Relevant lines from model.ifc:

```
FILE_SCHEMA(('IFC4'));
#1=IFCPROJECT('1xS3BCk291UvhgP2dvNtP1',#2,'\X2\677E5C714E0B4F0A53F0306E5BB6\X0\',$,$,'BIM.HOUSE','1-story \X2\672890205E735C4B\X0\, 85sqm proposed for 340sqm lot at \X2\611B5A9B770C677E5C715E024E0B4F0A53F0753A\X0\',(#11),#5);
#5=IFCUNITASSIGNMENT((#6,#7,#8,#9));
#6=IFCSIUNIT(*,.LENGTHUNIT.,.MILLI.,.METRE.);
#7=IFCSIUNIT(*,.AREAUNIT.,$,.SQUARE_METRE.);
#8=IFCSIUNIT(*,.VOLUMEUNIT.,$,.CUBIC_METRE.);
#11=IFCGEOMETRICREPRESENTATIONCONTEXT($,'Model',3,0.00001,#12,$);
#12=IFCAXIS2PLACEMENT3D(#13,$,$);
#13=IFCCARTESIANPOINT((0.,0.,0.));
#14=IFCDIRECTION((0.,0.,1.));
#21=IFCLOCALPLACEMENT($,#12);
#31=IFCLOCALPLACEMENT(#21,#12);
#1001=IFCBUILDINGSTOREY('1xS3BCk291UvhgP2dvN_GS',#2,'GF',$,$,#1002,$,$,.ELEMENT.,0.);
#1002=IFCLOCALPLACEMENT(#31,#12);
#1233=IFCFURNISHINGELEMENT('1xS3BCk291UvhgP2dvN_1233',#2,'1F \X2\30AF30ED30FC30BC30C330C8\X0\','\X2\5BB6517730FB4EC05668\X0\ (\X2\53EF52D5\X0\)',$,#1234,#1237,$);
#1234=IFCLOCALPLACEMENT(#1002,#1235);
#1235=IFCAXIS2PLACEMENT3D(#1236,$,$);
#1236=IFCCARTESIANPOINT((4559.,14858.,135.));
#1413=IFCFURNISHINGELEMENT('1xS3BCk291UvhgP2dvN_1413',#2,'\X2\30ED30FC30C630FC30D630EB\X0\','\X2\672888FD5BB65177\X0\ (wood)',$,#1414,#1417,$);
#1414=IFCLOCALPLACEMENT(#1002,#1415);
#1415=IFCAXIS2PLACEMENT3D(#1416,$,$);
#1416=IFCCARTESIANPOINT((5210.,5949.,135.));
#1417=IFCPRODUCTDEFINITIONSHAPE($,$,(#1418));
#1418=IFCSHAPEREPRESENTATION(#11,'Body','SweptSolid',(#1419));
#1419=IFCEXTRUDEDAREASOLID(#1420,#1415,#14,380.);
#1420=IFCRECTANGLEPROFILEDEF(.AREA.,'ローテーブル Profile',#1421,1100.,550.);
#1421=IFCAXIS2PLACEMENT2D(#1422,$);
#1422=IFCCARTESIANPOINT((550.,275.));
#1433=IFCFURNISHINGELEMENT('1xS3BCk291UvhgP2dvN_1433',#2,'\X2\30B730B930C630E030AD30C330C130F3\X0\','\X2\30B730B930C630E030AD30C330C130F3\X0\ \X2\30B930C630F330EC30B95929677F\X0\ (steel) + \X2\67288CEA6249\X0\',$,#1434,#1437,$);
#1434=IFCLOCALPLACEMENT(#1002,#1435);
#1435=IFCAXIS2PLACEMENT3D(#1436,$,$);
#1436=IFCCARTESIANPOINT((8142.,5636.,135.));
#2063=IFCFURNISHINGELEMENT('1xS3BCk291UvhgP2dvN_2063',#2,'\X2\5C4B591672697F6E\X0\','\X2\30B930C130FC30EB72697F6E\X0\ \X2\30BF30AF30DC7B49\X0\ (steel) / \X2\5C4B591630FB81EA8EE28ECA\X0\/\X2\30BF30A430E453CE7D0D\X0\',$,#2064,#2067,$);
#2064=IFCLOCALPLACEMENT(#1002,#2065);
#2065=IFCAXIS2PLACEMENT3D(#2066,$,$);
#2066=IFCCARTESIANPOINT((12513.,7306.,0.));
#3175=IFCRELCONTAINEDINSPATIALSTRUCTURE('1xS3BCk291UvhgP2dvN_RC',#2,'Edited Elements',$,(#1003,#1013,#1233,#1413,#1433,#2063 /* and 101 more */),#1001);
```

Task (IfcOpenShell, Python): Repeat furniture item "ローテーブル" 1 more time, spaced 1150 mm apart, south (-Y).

```python
import numpy as np
import ifcopenshell
import ifcopenshell.api.geometry
import ifcopenshell.api.root
import ifcopenshell.util.element
import ifcopenshell.util.placement
import ifcopenshell.util.unit

model = ifcopenshell.open("model.ifc")
unit_scale = ifcopenshell.util.unit.calculate_unit_scale(model)


def reuse_history(source, copy):
    """copy_class also copies each property set's owner history, people and application; keep the originals."""
    for rel in copy.IsDefinedBy:
        if rel.is_a("IfcRelDefinesByProperties") and (history := rel.RelatingPropertyDefinition.OwnerHistory):
            rel.RelatingPropertyDefinition.OwnerHistory = source.OwnerHistory
            ifcopenshell.util.element.remove_deep2(model, history)


source = model.by_guid("1xS3BCk291UvhgP2dvN_1413")
base = ifcopenshell.util.placement.get_local_placement(source.ObjectPlacement)
step = np.array([0.0, -1.0, 0.0]) * 1.15 / unit_scale

for i in range(1, 2):
    copy = ifcopenshell.api.root.copy_class(model, product=source)
    copy.Representation = ifcopenshell.util.element.copy_deep(
        model, source.Representation, exclude=["IfcGeometricRepresentationContext", "IfcRepresentationMap"]
    )
    reuse_history(source, copy)
    matrix = base.copy()
    matrix[:3, 3] += i * step
    print("added at", matrix[:3, 3].round(3) + 0.0)
    ifcopenshell.api.geometry.edit_object_placement(model, product=copy, matrix=matrix, is_si=False)

model.write("model_edited.ifc")
```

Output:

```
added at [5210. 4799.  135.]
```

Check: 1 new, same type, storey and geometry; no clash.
